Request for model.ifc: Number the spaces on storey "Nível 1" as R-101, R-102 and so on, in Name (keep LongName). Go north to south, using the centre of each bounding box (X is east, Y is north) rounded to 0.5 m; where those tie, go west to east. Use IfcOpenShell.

First a look at what the model holds.

```python
import ifcopenshell
import ifcopenshell.util.element
import ifcopenshell.util.placement

model = ifcopenshell.open("model.ifc")
print(model.schema)
storey = next(s for s in model.by_type("IfcBuildingStorey") if s.Name == "Nível 1")
spaces = [e for e in ifcopenshell.util.element.get_decomposition(storey) if e.is_a("IfcSpace")]
for e in sorted(spaces, key=lambda e: e.id()):
    origin = ifcopenshell.util.placement.get_local_placement(e.ObjectPlacement)[:3, 3]
    print(e.id(), e.Name, e.LongName, origin.round(2) + 0.0, sep=" | ")
```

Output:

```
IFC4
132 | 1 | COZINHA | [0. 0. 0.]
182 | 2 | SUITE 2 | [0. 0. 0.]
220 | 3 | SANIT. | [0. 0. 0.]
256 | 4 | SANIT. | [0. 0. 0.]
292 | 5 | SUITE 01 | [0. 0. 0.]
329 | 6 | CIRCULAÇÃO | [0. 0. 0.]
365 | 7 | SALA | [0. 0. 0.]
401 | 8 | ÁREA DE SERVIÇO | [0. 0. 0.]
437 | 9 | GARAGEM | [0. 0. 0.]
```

```python
import ifcopenshell
import ifcopenshell.geom
import ifcopenshell.util.element
import ifcopenshell.util.shape

model = ifcopenshell.open("model.ifc")
settings = ifcopenshell.geom.settings()
settings.set("use-world-coords", True)


def centre(element):
    shape = ifcopenshell.geom.create_shape(settings, element)
    return ifcopenshell.util.shape.get_bbox_centroid(shape.geometry)


storey = next(s for s in model.by_type("IfcBuildingStorey") if s.Name == "Nível 1")
spaces = [e for e in ifcopenshell.util.element.get_decomposition(storey) if e.is_a("IfcSpace")]

# Insertion points can sit at a corner or the storey origin, so sort by the geometry (in metres).
centres = {e: centre(e) for e in spaces}
spaces.sort(key=lambda e: (-round(centres[e][1] / 0.5), centres[e][0]))

for i, e in enumerate(spaces, start=1):
    number = f"R-1{i:02d}"
    e.Name = number
    print(e.id(), number)

model.write("model_rev.ifc")
```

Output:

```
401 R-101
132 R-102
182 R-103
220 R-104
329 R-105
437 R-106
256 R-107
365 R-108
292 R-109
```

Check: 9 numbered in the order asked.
